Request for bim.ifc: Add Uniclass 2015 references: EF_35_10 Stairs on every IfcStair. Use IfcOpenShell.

First a look at what the model holds.

```python
import ifcopenshell

model = ifcopenshell.open("bim.ifc")
print(model.schema)
print("classifications:", [c.Name for c in model.by_type("IfcClassification")])
for ifc_class in ("IfcDoor", "IfcRoof", "IfcStair", "IfcWall", "IfcWindow"):
    print(ifc_class, len(model.by_type(ifc_class)))
```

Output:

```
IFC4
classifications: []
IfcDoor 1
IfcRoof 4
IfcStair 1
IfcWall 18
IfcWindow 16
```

```python
import ifcopenshell
import ifcopenshell.api.classification

model = ifcopenshell.open("bim.ifc")

system = ifcopenshell.api.classification.add_classification(model, classification="Uniclass 2015")

codes = {
    "IfcStair": ("EF_35_10", "Stairs"),
}
for ifc_class, (code, name) in codes.items():
    products = model.by_type(ifc_class)
    ifcopenshell.api.classification.add_reference(
        model, products=products, classification=system, identification=code, name=name
    )
    print(code, len(products))

model.write("bim_v2.ifc")
```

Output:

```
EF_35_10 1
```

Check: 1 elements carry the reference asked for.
